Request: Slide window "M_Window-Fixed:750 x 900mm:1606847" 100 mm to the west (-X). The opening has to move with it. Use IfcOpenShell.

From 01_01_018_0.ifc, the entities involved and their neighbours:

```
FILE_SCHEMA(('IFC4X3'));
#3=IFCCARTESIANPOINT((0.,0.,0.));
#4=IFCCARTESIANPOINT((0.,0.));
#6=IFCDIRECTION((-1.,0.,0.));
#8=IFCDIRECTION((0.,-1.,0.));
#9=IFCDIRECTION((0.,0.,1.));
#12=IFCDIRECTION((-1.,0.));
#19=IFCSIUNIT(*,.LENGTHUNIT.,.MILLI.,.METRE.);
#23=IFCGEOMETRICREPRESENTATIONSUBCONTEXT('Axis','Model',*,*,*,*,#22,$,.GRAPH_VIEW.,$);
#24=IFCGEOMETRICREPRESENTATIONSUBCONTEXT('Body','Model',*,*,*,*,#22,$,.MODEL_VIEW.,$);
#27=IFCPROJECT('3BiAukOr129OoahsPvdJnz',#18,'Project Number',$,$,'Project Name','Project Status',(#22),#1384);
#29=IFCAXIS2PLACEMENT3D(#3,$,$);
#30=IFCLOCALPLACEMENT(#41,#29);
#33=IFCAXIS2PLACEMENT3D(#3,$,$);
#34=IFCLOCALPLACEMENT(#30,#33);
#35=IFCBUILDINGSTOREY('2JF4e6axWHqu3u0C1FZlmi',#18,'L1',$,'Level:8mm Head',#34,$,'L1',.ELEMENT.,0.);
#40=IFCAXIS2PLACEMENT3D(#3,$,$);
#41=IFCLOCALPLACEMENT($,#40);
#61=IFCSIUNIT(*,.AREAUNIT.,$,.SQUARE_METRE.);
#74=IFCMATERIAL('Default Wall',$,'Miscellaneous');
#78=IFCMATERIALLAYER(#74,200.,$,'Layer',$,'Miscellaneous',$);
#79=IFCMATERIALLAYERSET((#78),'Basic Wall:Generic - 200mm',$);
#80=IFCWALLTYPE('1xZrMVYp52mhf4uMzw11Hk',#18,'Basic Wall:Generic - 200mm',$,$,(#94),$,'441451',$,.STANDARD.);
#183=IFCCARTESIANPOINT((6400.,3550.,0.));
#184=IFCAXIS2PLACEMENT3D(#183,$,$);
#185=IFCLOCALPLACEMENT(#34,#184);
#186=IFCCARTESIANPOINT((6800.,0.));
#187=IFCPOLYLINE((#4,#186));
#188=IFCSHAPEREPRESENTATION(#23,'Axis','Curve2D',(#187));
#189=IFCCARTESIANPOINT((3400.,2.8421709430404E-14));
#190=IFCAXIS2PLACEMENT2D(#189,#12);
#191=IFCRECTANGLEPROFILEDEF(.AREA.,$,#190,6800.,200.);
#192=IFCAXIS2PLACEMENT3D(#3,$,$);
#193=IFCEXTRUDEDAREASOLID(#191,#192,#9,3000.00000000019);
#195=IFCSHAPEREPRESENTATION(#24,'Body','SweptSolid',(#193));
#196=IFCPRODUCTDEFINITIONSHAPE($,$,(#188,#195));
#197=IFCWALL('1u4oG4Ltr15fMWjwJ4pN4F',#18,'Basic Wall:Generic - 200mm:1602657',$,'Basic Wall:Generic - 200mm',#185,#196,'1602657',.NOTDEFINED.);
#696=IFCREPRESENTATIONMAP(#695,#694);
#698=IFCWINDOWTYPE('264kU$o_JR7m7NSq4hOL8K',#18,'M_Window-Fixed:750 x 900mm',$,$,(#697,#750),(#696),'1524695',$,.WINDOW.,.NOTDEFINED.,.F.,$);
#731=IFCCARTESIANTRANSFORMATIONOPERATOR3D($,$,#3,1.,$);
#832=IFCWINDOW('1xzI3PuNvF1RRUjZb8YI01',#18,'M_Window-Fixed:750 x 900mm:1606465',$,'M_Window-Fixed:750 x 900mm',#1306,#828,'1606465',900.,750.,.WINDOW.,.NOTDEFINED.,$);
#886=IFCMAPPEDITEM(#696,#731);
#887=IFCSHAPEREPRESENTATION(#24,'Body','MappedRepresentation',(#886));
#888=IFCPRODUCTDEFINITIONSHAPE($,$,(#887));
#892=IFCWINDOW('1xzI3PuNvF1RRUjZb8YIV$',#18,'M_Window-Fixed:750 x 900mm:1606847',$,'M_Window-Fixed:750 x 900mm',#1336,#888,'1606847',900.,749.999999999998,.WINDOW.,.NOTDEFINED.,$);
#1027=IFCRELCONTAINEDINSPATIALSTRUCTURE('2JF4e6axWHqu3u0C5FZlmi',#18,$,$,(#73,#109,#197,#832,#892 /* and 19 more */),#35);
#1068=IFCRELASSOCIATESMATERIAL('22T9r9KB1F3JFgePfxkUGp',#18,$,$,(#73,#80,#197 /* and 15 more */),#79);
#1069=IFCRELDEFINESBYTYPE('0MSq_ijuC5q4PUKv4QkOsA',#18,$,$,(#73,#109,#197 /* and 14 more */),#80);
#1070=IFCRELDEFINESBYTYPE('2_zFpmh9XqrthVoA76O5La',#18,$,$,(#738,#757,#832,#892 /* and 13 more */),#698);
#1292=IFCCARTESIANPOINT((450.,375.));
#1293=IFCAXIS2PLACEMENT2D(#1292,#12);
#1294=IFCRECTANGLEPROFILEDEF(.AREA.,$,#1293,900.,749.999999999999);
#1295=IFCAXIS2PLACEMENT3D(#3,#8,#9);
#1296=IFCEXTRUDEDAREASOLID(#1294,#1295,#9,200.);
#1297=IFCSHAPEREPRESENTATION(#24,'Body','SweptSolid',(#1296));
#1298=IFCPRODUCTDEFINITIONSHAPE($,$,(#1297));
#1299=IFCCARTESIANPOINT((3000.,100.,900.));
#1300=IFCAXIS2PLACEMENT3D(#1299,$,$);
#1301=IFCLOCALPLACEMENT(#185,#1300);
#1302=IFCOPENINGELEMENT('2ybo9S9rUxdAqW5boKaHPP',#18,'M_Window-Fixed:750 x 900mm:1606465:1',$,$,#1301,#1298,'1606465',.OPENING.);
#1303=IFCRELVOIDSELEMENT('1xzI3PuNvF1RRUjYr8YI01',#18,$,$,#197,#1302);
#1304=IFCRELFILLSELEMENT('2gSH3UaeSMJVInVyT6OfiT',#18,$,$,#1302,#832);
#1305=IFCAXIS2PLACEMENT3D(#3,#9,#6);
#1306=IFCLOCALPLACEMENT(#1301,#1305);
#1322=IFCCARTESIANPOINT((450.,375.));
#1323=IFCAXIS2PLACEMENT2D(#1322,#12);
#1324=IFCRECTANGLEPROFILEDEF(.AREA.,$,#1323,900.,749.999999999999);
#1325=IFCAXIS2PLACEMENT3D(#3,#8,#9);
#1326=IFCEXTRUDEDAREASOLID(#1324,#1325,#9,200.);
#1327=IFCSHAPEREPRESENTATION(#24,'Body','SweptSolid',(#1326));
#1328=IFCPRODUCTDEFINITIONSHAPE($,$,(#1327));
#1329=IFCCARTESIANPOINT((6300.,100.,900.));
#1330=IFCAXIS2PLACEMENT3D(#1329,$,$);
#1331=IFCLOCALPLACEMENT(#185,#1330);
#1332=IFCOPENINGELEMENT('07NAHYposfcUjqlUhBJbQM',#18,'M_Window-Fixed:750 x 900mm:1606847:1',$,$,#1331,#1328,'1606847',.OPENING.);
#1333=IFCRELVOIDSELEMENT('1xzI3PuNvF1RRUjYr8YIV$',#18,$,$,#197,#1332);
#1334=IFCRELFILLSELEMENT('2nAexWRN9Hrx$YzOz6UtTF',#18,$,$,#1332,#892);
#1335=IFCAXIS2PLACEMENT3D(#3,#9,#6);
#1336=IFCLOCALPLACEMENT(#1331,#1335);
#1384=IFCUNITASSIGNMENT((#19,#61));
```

```python
import ifcopenshell
import ifcopenshell.api.geometry
import ifcopenshell.util.placement
import ifcopenshell.util.unit

model = ifcopenshell.open("01_01_018_0.ifc")
unit_scale = ifcopenshell.util.unit.calculate_unit_scale(model)

window = model.by_id(892)
opening = window.FillsVoids[0].RelatingOpeningElement
wall = opening.VoidsElements[0].RelatingBuildingElement

wall_matrix = ifcopenshell.util.placement.get_local_placement(wall.ObjectPlacement)
shift = wall_matrix[:3, 0] * -0.1 / unit_scale
before = ifcopenshell.util.placement.get_local_placement(window.ObjectPlacement)[:3, 3].copy()

# The window is placed relative to its opening, so it follows when the opening moves.
matrix = ifcopenshell.util.placement.get_local_placement(opening.ObjectPlacement)
matrix[:3, 3] += shift
ifcopenshell.api.geometry.edit_object_placement(
    model, product=opening, matrix=matrix, is_si=False, should_transform_children=True
)

after = ifcopenshell.util.placement.get_local_placement(window.ObjectPlacement)[:3, 3]
print("window moved by", (after - before).round(3) + 0.0)

model.write("01_01_018_0_edited.ifc")
```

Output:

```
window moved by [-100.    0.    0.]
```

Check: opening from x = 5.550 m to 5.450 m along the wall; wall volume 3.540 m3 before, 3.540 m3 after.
